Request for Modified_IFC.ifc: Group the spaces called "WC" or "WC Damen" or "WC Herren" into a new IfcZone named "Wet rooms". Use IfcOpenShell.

First a look at what the model holds.

```python
import ifcopenshell

model = ifcopenshell.open("Modified_IFC.ifc")
print(model.schema)
seen = {}
for space in model.by_type("IfcSpace"):
    seen[space.LongName] = seen.get(space.LongName, 0) + 1
for name, count in sorted(seen.items(), key=str):
    print(count, "x", name)
print("zones:", [z.Name for z in model.by_type("IfcZone")][:20])
```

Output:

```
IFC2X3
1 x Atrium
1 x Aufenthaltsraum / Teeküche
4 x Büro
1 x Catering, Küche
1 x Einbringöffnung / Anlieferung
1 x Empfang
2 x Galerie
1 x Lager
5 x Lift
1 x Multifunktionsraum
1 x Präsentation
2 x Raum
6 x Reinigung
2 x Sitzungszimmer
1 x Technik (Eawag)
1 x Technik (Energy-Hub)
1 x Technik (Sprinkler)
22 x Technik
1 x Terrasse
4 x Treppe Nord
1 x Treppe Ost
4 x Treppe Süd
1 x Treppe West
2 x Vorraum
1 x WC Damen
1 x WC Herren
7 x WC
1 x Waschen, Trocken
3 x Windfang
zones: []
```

```python
import ifcopenshell
import ifcopenshell.api.group
import ifcopenshell.api.root

model = ifcopenshell.open("Modified_IFC.ifc")

names = {"WC", "WC Damen", "WC Herren"}
spaces = [s for s in model.by_type("IfcSpace") if s.LongName in names]

zone = ifcopenshell.api.root.create_entity(model, ifc_class="IfcZone", name="Wet rooms")
ifcopenshell.api.group.assign_group(model, products=spaces, group=zone)
print(len(spaces), "spaces in", zone.Name)

model.write("Modified_IFC_updated.ifc")
```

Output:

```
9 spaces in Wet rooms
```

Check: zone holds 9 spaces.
